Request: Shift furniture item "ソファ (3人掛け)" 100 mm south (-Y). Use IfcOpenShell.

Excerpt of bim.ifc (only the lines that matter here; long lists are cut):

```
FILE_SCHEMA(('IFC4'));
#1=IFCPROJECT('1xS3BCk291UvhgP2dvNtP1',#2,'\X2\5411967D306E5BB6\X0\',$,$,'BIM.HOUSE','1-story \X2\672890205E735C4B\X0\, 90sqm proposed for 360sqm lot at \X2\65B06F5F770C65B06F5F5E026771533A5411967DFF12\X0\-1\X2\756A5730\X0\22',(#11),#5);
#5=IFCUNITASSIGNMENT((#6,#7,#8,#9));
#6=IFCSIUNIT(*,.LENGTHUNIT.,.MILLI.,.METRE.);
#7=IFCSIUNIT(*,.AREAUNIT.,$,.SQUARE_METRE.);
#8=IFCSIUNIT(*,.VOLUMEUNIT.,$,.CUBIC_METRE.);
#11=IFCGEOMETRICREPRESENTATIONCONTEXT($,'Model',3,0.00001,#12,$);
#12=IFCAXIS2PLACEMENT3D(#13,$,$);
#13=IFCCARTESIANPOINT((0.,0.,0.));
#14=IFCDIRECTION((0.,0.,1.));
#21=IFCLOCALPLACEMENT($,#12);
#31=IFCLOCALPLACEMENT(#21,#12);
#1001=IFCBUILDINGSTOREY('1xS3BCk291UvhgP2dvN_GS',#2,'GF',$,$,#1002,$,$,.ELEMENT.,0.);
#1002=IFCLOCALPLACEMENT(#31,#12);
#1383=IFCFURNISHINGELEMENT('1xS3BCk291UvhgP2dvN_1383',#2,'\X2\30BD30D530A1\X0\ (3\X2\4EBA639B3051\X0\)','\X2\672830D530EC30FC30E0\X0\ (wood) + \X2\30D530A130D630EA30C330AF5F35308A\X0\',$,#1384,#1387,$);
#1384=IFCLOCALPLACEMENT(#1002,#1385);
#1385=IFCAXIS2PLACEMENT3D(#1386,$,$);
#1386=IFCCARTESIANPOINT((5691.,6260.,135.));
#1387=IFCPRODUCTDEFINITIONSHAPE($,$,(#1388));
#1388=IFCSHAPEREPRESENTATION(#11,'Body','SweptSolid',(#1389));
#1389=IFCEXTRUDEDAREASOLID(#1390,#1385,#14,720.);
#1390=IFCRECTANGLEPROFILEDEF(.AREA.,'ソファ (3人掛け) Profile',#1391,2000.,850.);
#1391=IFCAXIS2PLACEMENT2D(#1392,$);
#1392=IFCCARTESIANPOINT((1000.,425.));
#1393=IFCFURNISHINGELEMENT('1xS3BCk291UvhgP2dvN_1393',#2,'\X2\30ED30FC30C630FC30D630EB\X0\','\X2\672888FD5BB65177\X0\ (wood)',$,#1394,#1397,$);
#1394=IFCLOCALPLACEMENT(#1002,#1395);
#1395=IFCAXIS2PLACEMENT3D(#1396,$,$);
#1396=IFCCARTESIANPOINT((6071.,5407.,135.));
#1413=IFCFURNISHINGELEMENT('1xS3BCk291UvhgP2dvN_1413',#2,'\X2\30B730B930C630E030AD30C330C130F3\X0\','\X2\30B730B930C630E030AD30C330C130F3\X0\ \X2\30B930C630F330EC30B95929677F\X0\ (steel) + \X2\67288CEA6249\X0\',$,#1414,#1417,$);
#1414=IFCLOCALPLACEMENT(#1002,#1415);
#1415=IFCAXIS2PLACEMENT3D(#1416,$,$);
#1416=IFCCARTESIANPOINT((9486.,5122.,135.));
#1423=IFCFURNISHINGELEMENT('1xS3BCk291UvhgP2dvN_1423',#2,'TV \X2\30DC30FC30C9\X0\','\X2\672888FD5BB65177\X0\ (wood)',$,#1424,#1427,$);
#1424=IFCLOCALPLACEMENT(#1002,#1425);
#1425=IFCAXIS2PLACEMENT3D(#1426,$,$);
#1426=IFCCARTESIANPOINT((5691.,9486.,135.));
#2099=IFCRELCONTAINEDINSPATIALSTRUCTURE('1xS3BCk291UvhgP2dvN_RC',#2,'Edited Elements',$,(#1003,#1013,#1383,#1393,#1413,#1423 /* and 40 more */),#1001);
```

```python
import ifcopenshell
import ifcopenshell.api.geometry
import ifcopenshell.util.placement

model = ifcopenshell.open("bim.ifc")

item = model.by_guid("1xS3BCk291UvhgP2dvN_1383")
matrix = ifcopenshell.util.placement.get_local_placement(item.ObjectPlacement)
matrix[1, 3] -= 100.0
ifcopenshell.api.geometry.edit_object_placement(model, product=item, matrix=matrix, is_si=False)

print(ifcopenshell.util.placement.get_local_placement(item.ObjectPlacement).round(3) + 0.0)

model.write("bim_v2.ifc")
```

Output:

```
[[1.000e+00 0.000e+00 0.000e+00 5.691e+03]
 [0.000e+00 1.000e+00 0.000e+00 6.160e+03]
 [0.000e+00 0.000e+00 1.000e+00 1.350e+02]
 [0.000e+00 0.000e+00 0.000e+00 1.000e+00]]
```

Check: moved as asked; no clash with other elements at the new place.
